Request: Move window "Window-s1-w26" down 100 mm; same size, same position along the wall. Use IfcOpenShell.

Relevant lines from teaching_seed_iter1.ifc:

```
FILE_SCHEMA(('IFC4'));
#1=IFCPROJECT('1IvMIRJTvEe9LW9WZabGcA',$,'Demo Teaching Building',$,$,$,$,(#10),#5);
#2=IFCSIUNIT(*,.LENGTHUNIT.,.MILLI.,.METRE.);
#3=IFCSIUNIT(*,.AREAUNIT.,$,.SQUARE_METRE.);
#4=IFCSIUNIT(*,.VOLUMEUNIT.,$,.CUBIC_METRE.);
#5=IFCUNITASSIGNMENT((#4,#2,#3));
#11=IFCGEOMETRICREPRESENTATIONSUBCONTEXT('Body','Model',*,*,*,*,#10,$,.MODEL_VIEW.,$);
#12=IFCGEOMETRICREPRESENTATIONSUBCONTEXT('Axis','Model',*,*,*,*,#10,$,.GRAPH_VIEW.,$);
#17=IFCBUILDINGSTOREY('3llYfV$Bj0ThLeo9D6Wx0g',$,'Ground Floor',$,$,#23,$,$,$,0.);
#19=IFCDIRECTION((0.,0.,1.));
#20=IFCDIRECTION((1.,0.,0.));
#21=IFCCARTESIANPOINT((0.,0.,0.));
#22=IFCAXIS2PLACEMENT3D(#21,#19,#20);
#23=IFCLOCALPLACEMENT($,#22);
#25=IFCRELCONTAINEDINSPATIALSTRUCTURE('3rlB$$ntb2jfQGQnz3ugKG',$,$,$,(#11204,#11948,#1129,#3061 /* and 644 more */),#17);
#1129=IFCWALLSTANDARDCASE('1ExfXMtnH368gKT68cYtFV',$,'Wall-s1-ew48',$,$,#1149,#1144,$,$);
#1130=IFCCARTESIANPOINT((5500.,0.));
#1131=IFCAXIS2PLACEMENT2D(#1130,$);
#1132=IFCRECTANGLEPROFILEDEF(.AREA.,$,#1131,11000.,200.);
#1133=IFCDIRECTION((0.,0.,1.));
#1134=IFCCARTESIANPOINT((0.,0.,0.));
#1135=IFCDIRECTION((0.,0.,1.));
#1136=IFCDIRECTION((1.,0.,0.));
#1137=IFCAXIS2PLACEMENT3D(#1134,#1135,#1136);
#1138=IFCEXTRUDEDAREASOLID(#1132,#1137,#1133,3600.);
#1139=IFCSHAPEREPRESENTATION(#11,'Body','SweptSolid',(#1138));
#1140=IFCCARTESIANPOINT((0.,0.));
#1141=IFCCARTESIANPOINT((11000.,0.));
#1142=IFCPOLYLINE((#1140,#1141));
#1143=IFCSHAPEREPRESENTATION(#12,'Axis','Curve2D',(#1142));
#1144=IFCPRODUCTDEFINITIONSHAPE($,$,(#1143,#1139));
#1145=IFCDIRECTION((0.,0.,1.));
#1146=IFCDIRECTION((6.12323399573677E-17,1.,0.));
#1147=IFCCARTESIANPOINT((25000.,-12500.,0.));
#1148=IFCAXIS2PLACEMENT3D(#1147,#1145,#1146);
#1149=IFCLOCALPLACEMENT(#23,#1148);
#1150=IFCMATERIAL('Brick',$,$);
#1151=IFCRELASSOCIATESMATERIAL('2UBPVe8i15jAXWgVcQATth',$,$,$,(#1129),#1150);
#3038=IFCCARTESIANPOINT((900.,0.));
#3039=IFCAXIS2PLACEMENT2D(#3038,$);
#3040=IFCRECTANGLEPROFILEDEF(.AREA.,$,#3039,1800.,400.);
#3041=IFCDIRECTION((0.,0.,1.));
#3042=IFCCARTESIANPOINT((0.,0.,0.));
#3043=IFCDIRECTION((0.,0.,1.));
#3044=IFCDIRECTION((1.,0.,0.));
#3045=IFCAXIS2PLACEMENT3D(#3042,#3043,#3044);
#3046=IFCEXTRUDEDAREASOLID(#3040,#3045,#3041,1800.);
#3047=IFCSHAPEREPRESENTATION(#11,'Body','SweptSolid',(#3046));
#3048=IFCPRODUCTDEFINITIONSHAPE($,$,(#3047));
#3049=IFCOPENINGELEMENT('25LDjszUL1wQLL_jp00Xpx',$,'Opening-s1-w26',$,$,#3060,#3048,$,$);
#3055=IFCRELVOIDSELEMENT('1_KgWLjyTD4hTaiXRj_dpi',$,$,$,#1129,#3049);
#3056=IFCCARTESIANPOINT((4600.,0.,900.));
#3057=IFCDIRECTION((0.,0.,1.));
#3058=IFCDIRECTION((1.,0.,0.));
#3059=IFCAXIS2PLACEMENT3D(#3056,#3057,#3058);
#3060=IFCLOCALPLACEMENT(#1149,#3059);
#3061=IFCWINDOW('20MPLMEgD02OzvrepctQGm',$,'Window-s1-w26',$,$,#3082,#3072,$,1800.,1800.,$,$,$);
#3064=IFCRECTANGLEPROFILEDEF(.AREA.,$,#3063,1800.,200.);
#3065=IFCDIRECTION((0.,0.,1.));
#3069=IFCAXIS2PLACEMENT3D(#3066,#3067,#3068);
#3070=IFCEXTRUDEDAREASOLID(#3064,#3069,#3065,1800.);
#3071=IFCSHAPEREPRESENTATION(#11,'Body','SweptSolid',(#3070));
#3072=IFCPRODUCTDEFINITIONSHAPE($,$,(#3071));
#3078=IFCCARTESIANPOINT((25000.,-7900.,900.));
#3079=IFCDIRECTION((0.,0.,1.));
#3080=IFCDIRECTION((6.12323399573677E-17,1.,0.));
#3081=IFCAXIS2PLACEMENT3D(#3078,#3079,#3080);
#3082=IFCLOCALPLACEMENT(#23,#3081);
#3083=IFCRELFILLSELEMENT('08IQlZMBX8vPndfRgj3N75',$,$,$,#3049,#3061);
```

```python
import numpy as np
import ifcopenshell
import ifcopenshell.api.geometry
import ifcopenshell.util.placement
import ifcopenshell.util.unit

model = ifcopenshell.open("teaching_seed_iter1.ifc")
unit_scale = ifcopenshell.util.unit.calculate_unit_scale(model)

window = model.by_guid("20MPLMEgD02OzvrepctQGm")
opening = window.FillsVoids[0].RelatingOpeningElement
dz = -100.0

shift = np.array([0.0, 0.0, dz])
# The window is not placed relative to its opening, so move both.
for product in (opening, window):
    matrix = ifcopenshell.util.placement.get_local_placement(product.ObjectPlacement)
    matrix[:3, 3] += shift
    ifcopenshell.api.geometry.edit_object_placement(model, product=product, matrix=matrix, is_si=False)

print(f"moved by {dz * unit_scale:+.3f} m")

model.write("teaching_seed_iter1_rev.ifc")
```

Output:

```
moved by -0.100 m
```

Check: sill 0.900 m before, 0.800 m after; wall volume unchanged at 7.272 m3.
